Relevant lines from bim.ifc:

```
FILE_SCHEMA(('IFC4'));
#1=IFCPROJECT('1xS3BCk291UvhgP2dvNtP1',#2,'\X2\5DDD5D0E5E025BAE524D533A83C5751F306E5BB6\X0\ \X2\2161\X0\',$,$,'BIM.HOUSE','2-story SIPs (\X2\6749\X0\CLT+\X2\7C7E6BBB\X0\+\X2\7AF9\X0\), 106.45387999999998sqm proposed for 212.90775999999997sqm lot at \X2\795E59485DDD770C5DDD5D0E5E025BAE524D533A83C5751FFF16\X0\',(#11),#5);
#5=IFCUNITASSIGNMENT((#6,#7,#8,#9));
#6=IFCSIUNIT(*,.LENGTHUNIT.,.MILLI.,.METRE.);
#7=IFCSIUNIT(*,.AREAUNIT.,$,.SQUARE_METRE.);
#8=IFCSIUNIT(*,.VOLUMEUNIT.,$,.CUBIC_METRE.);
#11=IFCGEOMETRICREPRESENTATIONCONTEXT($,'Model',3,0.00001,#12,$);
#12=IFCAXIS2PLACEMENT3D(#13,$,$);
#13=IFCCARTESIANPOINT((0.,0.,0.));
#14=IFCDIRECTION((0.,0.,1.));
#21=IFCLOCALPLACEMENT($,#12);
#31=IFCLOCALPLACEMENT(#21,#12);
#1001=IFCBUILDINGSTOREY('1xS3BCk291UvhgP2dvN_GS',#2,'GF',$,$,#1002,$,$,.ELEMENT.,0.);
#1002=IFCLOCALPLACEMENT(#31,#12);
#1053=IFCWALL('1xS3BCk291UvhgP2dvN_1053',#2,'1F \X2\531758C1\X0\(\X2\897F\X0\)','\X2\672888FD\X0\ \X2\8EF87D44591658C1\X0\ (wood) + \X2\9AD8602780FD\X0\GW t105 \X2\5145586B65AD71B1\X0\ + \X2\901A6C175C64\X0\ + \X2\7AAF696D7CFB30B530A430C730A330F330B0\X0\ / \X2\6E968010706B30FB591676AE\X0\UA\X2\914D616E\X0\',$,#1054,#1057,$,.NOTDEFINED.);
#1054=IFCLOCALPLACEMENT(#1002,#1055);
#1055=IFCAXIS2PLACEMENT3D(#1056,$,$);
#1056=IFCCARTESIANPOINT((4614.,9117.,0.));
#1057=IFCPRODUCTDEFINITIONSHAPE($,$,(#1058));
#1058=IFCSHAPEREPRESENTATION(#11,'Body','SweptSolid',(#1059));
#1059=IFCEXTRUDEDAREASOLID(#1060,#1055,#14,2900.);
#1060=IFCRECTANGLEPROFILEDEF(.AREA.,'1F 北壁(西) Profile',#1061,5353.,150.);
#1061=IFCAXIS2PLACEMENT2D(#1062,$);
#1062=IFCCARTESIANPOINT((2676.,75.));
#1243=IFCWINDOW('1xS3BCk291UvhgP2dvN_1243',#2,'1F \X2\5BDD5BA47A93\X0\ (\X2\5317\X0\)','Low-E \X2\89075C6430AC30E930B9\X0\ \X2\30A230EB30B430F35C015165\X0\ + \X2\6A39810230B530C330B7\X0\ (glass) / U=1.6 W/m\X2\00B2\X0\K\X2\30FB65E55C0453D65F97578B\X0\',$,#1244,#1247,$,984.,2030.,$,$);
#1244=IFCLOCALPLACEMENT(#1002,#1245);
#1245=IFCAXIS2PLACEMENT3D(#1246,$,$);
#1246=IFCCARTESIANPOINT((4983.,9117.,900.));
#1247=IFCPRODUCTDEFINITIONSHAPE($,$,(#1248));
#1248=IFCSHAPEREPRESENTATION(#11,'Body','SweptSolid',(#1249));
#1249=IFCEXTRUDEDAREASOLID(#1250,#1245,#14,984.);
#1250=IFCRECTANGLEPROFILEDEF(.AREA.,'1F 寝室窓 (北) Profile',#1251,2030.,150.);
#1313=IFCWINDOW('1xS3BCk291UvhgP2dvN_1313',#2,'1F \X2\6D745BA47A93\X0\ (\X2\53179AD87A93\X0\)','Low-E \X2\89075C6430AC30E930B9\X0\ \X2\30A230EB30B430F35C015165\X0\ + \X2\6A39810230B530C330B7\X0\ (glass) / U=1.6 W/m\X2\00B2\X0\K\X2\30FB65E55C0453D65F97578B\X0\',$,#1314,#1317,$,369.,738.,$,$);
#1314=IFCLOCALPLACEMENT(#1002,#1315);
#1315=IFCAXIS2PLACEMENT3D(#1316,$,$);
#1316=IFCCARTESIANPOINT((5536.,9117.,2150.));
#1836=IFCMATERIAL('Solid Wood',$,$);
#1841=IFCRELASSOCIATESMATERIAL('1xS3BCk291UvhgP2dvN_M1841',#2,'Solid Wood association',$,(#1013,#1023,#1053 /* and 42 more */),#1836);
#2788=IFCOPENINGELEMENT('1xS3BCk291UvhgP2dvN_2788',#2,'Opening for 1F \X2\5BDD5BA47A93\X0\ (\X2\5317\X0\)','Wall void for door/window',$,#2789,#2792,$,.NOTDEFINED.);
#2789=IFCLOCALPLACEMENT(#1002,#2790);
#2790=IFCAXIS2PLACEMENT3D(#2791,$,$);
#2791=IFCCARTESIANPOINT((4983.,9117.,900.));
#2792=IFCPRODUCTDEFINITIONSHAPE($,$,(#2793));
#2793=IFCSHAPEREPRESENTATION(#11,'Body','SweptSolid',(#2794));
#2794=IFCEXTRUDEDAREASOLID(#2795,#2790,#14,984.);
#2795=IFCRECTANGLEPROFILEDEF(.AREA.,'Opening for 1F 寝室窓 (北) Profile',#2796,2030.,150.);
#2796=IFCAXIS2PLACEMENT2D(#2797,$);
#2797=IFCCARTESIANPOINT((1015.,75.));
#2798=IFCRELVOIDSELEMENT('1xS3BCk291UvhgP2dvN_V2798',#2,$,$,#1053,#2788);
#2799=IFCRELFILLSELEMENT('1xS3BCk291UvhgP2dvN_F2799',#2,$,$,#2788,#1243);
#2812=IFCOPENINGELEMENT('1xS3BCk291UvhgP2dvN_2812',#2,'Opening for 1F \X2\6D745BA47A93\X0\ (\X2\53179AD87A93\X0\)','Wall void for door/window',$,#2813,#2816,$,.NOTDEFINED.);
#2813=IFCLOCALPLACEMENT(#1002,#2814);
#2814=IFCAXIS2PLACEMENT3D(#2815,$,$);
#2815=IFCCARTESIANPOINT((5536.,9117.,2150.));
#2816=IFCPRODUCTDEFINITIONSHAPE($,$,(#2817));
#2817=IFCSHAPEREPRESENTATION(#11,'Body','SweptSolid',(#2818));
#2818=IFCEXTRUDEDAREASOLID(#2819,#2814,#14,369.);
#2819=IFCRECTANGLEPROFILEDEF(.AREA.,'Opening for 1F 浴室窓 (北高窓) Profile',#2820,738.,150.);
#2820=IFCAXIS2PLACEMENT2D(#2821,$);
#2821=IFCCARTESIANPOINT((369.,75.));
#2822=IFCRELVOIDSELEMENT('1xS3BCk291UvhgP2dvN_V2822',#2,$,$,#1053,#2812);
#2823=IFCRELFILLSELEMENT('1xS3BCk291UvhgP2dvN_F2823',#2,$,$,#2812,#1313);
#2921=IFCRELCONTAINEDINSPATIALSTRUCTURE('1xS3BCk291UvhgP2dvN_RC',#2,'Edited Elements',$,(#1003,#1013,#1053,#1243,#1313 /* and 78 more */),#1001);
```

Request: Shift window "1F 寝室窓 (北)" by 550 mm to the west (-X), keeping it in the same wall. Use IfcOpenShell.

```python
import ifcopenshell
import ifcopenshell.api.geometry
import ifcopenshell.util.placement

model = ifcopenshell.open("bim.ifc")

window = model.by_guid("1xS3BCk291UvhgP2dvN_1243")
opening = window.FillsVoids[0].RelatingOpeningElement
wall = opening.VoidsElements[0].RelatingBuildingElement

wall_matrix = ifcopenshell.util.placement.get_local_placement(wall.ObjectPlacement)
shift = wall_matrix[:3, 0] * -550.0
before = ifcopenshell.util.placement.get_local_placement(window.ObjectPlacement)[:3, 3].copy()

# The window is not placed relative to its opening, so move both.
for product in (opening, window):
    matrix = ifcopenshell.util.placement.get_local_placement(product.ObjectPlacement)
    matrix[:3, 3] += shift
    ifcopenshell.api.geometry.edit_object_placement(model, product=product, matrix=matrix, is_si=False)

after = ifcopenshell.util.placement.get_local_placement(window.ObjectPlacement)[:3, 3]
print("window moved by", (after - before).round(3) + 0.0)

model.write("bim_edited.ifc")
```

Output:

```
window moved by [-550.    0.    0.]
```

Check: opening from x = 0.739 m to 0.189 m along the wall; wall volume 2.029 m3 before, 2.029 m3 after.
